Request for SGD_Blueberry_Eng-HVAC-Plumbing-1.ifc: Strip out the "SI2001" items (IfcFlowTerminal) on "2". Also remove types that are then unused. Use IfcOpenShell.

First a look at what the model holds.

```python
import ifcopenshell
import ifcopenshell.util.element

model = ifcopenshell.open("SGD_Blueberry_Eng-HVAC-Plumbing-1.ifc")
print(model.schema)
storey = next(s for s in model.by_type("IfcBuildingStorey") if s.Name == "2")
terminals = [e for e in ifcopenshell.util.element.get_decomposition(storey) if e.is_a("IfcFlowTerminal")]
seen = {}
for e in terminals:
    element_type = ifcopenshell.util.element.get_type(e)
    name = element_type.Name if element_type not in (None, e) else None
    seen[name] = seen.get(name, 0) + 1
for name, count in sorted(seen.items(), key=str):
    print(count, "x", name)
```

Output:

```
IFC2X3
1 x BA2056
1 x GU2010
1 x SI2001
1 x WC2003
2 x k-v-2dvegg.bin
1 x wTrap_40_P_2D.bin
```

```python
import ifcopenshell
import ifcopenshell.api.root
import ifcopenshell.util.element

model = ifcopenshell.open("SGD_Blueberry_Eng-HVAC-Plumbing-1.ifc")

storey = next(s for s in model.by_type("IfcBuildingStorey") if s.Name == "2")
terminals = [e for e in ifcopenshell.util.element.get_decomposition(storey) if e.is_a("IfcFlowTerminal")]
targets = [e for e in terminals if (t := ifcopenshell.util.element.get_type(e)) not in (None, e) and t.Name == "SI2001"]
types = {ifcopenshell.util.element.get_type(e) for e in targets} - {None, *targets}

for e in targets:
    ifcopenshell.api.root.remove_product(model, product=e)
print(len(targets), "removed")

unused = [t for t in types if not ifcopenshell.util.element.get_types(t)]
for t in unused:
    ifcopenshell.api.root.remove_product(model, product=t)
print(len(unused), "unused types removed")

model.write("SGD_Blueberry_Eng-HVAC-Plumbing-1-out.ifc")
```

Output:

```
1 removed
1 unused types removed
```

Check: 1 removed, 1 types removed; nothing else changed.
